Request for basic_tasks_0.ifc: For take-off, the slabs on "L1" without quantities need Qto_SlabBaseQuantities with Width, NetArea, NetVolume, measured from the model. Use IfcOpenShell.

First a look at what the model holds.

```python
import ifcopenshell
import ifcopenshell.util.element
import ifcopenshell.util.unit

model = ifcopenshell.open("basic_tasks_0.ifc")
print(model.schema)
for unit_type in ("LENGTHUNIT", "AREAUNIT", "VOLUMEUNIT"):
    print(unit_type, ifcopenshell.util.unit.calculate_unit_scale(model, unit_type))
storey = next(s for s in model.by_type("IfcBuildingStorey") if s.Name == "L1")
slabs = [e for e in ifcopenshell.util.element.get_decomposition(storey) if e.is_a("IfcSlab")]
for e in sorted(slabs, key=lambda e: e.id()):
    print(e.id(), e.is_a(), e.Name, list(ifcopenshell.util.element.get_psets(e, qtos_only=True)), sep=" | ")
```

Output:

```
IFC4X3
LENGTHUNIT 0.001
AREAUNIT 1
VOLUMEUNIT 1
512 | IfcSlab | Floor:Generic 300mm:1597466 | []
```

```python
import ifcopenshell
import ifcopenshell.api.pset
import ifcopenshell.geom
import ifcopenshell.util.element
import ifcopenshell.util.shape
import ifcopenshell.util.unit

model = ifcopenshell.open("basic_tasks_0.ifc")
unit_scale = ifcopenshell.util.unit.calculate_unit_scale(model)
area_scale = ifcopenshell.util.unit.calculate_unit_scale(model, "AREAUNIT")
volume_scale = ifcopenshell.util.unit.calculate_unit_scale(model, "VOLUMEUNIT")
settings = ifcopenshell.geom.settings()

storey = next(s for s in model.by_type("IfcBuildingStorey") if s.Name == "L1")
slabs = [e for e in ifcopenshell.util.element.get_decomposition(storey) if e.is_a("IfcSlab")]

for e in sorted(slabs, key=lambda e: e.id()):
    if ifcopenshell.util.element.get_psets(e, qtos_only=True, should_inherit=False):
        continue
    # Geometry comes back in metres, in the element's own axes.
    shape = ifcopenshell.geom.create_shape(settings, e)
    values = {
        "Width": ifcopenshell.util.shape.get_z(shape.geometry) / unit_scale,
        "NetArea": ifcopenshell.util.shape.get_footprint_area(shape.geometry) / area_scale,
        "NetVolume": ifcopenshell.util.shape.get_volume(shape.geometry) / volume_scale,
    }
    qto = ifcopenshell.api.pset.add_qto(model, product=e, name="Qto_SlabBaseQuantities")
    ifcopenshell.api.pset.edit_qto(model, qto=qto, properties=values)
    print(e.id(), {k: round(v, 3) for k, v in values.items()})

model.write("basic_tasks_0_v2.ifc")
```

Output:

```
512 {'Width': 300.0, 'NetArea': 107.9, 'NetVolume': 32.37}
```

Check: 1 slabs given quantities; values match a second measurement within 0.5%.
